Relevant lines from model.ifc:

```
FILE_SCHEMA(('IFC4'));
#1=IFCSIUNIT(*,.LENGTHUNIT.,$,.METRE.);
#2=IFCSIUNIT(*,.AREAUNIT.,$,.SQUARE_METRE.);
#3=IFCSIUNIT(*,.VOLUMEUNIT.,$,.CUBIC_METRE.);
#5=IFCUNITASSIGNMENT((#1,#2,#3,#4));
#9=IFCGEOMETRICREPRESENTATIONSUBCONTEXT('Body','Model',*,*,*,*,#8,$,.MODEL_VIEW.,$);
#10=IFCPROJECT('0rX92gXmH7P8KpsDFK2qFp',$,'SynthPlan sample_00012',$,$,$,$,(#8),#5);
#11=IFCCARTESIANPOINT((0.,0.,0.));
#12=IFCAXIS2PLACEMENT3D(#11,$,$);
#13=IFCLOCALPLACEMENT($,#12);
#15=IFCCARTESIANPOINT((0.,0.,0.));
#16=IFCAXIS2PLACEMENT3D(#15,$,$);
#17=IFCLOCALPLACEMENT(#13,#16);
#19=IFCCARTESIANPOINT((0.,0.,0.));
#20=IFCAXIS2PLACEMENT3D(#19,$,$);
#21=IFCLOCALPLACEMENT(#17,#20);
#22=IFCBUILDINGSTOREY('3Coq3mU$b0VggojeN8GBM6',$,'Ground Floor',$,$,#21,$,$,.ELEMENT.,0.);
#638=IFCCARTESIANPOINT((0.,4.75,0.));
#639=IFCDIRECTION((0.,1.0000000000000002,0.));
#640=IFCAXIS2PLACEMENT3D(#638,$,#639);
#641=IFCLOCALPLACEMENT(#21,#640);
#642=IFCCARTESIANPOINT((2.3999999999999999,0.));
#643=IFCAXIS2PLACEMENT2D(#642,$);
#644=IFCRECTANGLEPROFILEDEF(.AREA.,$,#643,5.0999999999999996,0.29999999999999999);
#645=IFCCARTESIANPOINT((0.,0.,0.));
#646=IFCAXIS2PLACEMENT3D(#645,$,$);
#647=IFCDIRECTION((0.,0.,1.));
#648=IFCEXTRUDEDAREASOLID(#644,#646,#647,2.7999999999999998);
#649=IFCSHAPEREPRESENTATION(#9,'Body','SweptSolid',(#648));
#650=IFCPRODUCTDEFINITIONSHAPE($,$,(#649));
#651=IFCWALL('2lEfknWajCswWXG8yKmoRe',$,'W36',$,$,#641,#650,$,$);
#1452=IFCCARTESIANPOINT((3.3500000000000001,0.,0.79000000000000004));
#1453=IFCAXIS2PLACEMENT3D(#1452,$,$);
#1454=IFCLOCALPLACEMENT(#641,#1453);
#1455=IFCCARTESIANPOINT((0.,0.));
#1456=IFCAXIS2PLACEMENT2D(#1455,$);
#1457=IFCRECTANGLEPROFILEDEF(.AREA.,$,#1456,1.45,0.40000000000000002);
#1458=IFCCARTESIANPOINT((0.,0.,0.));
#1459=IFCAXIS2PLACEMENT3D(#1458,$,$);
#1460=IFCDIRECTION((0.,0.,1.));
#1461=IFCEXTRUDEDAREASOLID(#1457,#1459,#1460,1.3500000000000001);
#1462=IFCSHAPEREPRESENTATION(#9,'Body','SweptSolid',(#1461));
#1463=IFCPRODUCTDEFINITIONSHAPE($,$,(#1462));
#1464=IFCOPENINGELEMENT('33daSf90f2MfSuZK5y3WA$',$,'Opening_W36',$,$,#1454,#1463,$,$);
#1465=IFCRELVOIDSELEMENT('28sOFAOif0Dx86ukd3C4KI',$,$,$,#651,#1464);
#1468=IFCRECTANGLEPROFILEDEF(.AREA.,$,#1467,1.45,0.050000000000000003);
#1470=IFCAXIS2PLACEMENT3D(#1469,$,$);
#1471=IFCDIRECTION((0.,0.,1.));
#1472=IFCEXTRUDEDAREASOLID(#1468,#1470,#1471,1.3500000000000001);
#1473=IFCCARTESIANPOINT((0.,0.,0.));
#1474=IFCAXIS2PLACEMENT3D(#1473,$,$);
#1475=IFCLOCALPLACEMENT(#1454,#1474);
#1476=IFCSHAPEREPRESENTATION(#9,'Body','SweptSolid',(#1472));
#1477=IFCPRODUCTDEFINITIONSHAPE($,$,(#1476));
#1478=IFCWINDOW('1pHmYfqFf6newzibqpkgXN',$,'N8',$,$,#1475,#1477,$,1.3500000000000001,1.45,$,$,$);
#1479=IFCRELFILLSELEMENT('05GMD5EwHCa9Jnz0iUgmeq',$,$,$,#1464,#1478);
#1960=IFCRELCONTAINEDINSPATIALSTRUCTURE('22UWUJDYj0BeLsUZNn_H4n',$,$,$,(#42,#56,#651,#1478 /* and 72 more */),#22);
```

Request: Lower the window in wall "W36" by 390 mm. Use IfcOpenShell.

```python
import numpy as np
import ifcopenshell
import ifcopenshell.api.geometry
import ifcopenshell.util.placement
import ifcopenshell.util.unit

model = ifcopenshell.open("model.ifc")
unit_scale = ifcopenshell.util.unit.calculate_unit_scale(model)

window = model.by_id(1478)
opening = window.FillsVoids[0].RelatingOpeningElement
dz = -0.39

shift = np.array([0.0, 0.0, dz])
# The window is placed relative to its opening, so it follows when the opening moves.
matrix = ifcopenshell.util.placement.get_local_placement(opening.ObjectPlacement)
matrix[:3, 3] += shift
ifcopenshell.api.geometry.edit_object_placement(
    model, product=opening, matrix=matrix, is_si=False, should_transform_children=True
)

print(f"moved by {dz * unit_scale:+.3f} m")

model.write("model_edited.ifc")
```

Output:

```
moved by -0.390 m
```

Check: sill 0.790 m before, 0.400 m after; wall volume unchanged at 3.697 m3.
